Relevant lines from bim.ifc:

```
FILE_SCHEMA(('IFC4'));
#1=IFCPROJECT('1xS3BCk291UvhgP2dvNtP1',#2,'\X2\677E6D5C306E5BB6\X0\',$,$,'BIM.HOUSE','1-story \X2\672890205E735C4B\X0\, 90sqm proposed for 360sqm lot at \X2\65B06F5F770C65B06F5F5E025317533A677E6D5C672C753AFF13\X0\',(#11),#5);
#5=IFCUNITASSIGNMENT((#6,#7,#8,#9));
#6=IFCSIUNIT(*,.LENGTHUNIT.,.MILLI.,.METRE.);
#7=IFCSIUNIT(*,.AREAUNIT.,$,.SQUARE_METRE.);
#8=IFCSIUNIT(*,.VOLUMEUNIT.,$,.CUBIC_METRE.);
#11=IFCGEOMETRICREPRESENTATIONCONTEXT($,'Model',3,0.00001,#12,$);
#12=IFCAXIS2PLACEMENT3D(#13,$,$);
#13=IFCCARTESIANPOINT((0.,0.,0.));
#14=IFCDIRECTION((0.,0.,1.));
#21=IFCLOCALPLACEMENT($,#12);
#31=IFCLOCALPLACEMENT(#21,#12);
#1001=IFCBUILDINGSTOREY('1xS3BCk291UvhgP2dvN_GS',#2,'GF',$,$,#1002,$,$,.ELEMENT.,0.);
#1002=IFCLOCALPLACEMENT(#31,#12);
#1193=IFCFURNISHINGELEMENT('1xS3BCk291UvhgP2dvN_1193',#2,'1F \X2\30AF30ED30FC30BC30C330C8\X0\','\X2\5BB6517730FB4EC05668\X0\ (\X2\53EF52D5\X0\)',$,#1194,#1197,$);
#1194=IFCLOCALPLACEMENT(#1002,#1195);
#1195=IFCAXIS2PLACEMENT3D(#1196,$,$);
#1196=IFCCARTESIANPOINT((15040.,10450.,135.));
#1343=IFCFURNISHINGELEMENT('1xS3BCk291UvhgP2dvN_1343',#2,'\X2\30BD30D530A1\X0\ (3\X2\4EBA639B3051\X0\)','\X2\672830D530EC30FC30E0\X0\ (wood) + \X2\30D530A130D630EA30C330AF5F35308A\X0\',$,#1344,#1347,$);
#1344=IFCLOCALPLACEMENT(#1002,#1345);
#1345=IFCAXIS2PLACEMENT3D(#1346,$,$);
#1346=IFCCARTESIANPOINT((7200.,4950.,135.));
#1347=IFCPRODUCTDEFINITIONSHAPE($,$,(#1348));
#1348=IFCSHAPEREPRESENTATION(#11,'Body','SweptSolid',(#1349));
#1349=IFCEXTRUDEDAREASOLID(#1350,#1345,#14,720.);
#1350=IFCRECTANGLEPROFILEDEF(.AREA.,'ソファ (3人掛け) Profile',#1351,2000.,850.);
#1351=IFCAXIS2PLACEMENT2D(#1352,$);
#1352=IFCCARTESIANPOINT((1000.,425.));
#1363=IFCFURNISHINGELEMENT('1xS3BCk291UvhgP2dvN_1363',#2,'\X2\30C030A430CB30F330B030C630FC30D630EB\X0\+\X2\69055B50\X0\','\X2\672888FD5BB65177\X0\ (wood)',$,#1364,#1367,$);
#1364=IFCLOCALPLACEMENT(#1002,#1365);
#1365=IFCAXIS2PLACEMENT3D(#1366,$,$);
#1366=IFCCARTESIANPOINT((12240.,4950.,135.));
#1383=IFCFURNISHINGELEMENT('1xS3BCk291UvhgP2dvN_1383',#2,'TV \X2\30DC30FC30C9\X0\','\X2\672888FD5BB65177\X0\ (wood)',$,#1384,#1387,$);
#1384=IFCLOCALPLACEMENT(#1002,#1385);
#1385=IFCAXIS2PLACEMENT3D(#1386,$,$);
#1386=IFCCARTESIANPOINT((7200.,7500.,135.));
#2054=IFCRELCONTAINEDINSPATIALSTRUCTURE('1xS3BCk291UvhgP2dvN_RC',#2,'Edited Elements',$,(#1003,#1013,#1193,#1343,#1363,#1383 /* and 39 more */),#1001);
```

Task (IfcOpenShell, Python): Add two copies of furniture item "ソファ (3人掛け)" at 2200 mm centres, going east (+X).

```python
import numpy as np
import ifcopenshell
import ifcopenshell.api.geometry
import ifcopenshell.api.root
import ifcopenshell.util.element
import ifcopenshell.util.placement

model = ifcopenshell.open("bim.ifc")


def reuse_history(source, copy):
    """copy_class also copies each property set's owner history, people and application; keep the originals."""
    for rel in copy.IsDefinedBy:
        if rel.is_a("IfcRelDefinesByProperties") and (history := rel.RelatingPropertyDefinition.OwnerHistory):
            rel.RelatingPropertyDefinition.OwnerHistory = source.OwnerHistory
            ifcopenshell.util.element.remove_deep2(model, history)


source = model.by_id(1343)
base = ifcopenshell.util.placement.get_local_placement(source.ObjectPlacement)
step = np.array([1.0, 0.0, 0.0]) * 2200.0

for i in range(1, 3):
    copy = ifcopenshell.api.root.copy_class(model, product=source)
    copy.Representation = ifcopenshell.util.element.copy_deep(
        model, source.Representation, exclude=["IfcGeometricRepresentationContext", "IfcRepresentationMap"]
    )
    reuse_history(source, copy)
    matrix = base.copy()
    matrix[:3, 3] += i * step
    print("added at", matrix[:3, 3].round(3) + 0.0)
    ifcopenshell.api.geometry.edit_object_placement(model, product=copy, matrix=matrix, is_si=False)

model.write("bim_v2.ifc")
```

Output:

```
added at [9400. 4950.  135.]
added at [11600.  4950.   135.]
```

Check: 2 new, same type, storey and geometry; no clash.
